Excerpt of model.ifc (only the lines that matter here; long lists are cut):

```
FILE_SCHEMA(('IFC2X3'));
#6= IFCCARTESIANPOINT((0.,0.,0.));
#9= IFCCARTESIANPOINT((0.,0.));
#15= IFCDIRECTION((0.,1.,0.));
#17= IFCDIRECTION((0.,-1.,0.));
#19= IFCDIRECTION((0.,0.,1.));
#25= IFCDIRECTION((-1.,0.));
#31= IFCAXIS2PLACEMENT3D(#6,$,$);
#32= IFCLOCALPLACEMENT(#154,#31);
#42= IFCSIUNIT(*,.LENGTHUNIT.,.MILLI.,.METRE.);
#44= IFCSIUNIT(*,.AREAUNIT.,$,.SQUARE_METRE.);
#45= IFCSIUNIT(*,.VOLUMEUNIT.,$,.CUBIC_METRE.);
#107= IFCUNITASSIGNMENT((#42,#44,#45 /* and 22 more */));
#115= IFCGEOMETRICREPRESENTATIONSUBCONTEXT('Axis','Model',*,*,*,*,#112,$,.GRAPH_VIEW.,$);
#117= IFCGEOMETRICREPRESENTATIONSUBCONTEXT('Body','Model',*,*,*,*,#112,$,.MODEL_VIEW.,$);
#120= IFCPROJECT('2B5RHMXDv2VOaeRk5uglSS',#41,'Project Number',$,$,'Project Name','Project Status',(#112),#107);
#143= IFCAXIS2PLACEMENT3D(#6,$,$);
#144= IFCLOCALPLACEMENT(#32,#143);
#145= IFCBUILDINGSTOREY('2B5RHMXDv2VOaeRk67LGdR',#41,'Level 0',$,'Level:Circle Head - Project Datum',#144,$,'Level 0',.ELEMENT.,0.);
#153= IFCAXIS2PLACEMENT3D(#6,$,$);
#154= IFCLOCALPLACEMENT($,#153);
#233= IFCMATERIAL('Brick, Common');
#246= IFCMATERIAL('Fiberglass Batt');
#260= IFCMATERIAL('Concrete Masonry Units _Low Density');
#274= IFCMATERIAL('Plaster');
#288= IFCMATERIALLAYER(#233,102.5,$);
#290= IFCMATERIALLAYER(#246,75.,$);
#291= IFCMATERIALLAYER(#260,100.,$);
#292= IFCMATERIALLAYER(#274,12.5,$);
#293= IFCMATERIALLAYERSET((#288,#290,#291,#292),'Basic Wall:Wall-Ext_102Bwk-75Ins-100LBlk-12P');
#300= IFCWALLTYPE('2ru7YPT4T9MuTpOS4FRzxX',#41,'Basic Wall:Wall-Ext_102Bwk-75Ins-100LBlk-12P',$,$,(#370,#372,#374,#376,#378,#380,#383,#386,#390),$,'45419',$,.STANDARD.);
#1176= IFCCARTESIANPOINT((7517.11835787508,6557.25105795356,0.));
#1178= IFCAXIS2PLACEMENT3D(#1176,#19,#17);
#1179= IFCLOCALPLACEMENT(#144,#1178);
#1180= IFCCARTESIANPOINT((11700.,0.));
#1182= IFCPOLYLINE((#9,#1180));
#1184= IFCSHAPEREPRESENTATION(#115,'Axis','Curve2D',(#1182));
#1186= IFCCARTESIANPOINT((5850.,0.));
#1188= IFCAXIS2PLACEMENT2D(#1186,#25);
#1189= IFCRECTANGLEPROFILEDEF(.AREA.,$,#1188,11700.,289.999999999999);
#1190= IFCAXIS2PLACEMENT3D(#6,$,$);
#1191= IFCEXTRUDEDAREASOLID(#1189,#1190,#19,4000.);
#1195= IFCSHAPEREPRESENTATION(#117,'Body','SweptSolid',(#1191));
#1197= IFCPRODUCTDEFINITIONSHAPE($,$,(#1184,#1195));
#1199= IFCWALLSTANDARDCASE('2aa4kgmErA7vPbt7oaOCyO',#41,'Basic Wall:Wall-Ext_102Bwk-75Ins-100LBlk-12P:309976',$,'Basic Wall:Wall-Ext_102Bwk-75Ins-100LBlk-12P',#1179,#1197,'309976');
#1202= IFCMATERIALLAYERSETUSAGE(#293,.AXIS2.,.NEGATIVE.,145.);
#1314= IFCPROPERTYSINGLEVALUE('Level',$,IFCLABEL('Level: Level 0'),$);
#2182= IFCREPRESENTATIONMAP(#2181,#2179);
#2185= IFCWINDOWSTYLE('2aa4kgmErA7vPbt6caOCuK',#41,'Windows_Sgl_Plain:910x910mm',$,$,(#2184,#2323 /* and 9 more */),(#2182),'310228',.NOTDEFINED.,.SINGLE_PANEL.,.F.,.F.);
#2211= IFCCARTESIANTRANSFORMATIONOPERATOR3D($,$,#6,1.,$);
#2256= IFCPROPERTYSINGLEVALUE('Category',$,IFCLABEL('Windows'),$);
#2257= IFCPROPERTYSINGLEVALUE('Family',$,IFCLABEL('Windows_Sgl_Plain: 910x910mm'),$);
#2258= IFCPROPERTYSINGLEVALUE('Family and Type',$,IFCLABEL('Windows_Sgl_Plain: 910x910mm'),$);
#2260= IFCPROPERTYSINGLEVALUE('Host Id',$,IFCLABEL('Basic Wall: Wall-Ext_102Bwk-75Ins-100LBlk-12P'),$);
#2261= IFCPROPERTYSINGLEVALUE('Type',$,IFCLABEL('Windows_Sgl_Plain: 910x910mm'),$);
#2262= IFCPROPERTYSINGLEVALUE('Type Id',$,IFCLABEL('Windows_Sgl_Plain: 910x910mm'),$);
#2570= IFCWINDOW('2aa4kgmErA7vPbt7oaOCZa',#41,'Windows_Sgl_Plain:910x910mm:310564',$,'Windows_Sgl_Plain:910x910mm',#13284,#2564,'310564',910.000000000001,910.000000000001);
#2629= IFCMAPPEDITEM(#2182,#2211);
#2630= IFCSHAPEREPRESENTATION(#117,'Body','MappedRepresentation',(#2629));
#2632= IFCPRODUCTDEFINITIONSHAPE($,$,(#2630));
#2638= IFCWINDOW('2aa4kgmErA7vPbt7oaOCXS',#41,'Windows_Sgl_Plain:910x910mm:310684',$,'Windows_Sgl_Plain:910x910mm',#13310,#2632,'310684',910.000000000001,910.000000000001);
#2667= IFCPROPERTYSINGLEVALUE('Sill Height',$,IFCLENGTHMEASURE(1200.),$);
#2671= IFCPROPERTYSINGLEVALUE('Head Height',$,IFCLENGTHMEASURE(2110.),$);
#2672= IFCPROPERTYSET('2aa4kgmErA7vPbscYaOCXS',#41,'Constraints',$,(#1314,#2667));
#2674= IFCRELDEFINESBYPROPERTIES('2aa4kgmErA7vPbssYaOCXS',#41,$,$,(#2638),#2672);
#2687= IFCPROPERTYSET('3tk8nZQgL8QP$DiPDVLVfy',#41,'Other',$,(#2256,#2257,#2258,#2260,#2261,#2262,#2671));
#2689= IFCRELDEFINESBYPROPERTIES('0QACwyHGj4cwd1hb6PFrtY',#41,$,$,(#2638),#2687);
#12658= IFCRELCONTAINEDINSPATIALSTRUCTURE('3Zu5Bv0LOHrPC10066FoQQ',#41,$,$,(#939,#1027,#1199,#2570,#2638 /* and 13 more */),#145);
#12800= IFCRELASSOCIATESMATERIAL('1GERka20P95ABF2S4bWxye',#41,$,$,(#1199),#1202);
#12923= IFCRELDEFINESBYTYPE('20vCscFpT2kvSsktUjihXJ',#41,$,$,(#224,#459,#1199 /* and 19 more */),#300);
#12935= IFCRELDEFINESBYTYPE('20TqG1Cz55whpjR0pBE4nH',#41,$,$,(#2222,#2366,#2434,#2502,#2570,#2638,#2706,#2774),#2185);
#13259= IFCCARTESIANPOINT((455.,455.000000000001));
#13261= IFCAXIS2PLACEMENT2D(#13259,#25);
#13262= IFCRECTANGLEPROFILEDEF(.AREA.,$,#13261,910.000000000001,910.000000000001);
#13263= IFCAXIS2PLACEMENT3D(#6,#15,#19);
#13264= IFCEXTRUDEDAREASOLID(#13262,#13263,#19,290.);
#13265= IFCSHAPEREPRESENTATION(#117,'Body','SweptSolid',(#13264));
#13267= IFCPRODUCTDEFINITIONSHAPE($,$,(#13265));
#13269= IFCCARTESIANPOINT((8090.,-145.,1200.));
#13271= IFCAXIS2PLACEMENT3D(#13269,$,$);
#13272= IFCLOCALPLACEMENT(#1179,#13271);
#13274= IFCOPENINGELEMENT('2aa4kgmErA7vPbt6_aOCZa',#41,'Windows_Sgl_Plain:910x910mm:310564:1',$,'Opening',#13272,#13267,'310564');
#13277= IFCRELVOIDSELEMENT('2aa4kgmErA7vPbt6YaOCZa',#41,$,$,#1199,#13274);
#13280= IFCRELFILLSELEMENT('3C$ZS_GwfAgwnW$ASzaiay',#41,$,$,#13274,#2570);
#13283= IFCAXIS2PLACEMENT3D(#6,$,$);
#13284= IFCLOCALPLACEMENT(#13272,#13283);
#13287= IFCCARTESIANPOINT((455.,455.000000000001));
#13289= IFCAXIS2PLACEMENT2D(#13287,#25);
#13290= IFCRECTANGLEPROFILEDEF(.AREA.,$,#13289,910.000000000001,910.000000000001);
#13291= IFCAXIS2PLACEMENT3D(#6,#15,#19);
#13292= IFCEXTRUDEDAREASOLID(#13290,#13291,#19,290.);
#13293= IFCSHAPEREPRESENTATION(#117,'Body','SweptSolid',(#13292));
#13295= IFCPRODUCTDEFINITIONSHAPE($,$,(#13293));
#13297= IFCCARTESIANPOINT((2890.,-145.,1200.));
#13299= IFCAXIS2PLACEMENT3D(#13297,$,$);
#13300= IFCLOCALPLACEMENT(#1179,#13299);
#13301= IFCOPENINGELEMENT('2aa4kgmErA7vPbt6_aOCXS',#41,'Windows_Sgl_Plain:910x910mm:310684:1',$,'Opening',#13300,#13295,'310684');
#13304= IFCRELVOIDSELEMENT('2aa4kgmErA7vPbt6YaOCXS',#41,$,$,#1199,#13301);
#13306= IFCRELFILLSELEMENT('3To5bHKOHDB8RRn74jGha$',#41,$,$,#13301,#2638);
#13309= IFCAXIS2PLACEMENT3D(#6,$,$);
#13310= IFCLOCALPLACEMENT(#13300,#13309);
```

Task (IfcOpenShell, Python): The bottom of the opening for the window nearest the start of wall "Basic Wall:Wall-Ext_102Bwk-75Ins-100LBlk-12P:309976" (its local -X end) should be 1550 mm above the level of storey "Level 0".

```python
import numpy as np
import ifcopenshell
import ifcopenshell.api.geometry
import ifcopenshell.api.pset
import ifcopenshell.geom
import ifcopenshell.util.element
import ifcopenshell.util.placement
import ifcopenshell.util.shape
import ifcopenshell.util.unit

model = ifcopenshell.open("model.ifc")
unit_scale = ifcopenshell.util.unit.calculate_unit_scale(model)

window = model.by_id(2638)
opening = window.FillsVoids[0].RelatingOpeningElement
storey = ifcopenshell.util.element.get_container(window, ifc_class="IfcBuildingStorey")
level = ifcopenshell.util.placement.get_local_placement(storey.ObjectPlacement)[2, 3]

# The opening's origin need not be at the sill, so measure its lowest point.
shape = ifcopenshell.geom.create_shape(ifcopenshell.geom.settings(), opening)
bottom = ifcopenshell.util.shape.get_shape_bottom_elevation(shape, shape.geometry) / unit_scale
dz = level + 1.55 / unit_scale - bottom

shift = np.array([0.0, 0.0, dz])
# The window is placed relative to its opening, so it follows when the opening moves.
matrix = ifcopenshell.util.placement.get_local_placement(opening.ObjectPlacement)
matrix[:3, 3] += shift
ifcopenshell.api.geometry.edit_object_placement(
    model, product=opening, matrix=matrix, is_si=False, should_transform_children=True
)

# Keep the stored heights in step.
pset = model.by_id(ifcopenshell.util.element.get_pset(window, "Constraints", should_inherit=False)["id"])
ifcopenshell.api.pset.edit_pset(model, pset=pset, properties={
    "Sill Height": model.create_entity("IfcLengthMeasure", ifcopenshell.util.element.get_pset(window, "Constraints", "Sill Height") + dz),
})
pset = model.by_id(ifcopenshell.util.element.get_pset(window, "Other", should_inherit=False)["id"])
ifcopenshell.api.pset.edit_pset(model, pset=pset, properties={
    "Head Height": model.create_entity("IfcLengthMeasure", ifcopenshell.util.element.get_pset(window, "Other", "Head Height") + dz),
})

print(f"moved by {dz * unit_scale:+.3f} m")

model.write("model_rev.ifc")
```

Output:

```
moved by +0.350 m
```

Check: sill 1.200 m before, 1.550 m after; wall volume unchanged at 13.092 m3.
